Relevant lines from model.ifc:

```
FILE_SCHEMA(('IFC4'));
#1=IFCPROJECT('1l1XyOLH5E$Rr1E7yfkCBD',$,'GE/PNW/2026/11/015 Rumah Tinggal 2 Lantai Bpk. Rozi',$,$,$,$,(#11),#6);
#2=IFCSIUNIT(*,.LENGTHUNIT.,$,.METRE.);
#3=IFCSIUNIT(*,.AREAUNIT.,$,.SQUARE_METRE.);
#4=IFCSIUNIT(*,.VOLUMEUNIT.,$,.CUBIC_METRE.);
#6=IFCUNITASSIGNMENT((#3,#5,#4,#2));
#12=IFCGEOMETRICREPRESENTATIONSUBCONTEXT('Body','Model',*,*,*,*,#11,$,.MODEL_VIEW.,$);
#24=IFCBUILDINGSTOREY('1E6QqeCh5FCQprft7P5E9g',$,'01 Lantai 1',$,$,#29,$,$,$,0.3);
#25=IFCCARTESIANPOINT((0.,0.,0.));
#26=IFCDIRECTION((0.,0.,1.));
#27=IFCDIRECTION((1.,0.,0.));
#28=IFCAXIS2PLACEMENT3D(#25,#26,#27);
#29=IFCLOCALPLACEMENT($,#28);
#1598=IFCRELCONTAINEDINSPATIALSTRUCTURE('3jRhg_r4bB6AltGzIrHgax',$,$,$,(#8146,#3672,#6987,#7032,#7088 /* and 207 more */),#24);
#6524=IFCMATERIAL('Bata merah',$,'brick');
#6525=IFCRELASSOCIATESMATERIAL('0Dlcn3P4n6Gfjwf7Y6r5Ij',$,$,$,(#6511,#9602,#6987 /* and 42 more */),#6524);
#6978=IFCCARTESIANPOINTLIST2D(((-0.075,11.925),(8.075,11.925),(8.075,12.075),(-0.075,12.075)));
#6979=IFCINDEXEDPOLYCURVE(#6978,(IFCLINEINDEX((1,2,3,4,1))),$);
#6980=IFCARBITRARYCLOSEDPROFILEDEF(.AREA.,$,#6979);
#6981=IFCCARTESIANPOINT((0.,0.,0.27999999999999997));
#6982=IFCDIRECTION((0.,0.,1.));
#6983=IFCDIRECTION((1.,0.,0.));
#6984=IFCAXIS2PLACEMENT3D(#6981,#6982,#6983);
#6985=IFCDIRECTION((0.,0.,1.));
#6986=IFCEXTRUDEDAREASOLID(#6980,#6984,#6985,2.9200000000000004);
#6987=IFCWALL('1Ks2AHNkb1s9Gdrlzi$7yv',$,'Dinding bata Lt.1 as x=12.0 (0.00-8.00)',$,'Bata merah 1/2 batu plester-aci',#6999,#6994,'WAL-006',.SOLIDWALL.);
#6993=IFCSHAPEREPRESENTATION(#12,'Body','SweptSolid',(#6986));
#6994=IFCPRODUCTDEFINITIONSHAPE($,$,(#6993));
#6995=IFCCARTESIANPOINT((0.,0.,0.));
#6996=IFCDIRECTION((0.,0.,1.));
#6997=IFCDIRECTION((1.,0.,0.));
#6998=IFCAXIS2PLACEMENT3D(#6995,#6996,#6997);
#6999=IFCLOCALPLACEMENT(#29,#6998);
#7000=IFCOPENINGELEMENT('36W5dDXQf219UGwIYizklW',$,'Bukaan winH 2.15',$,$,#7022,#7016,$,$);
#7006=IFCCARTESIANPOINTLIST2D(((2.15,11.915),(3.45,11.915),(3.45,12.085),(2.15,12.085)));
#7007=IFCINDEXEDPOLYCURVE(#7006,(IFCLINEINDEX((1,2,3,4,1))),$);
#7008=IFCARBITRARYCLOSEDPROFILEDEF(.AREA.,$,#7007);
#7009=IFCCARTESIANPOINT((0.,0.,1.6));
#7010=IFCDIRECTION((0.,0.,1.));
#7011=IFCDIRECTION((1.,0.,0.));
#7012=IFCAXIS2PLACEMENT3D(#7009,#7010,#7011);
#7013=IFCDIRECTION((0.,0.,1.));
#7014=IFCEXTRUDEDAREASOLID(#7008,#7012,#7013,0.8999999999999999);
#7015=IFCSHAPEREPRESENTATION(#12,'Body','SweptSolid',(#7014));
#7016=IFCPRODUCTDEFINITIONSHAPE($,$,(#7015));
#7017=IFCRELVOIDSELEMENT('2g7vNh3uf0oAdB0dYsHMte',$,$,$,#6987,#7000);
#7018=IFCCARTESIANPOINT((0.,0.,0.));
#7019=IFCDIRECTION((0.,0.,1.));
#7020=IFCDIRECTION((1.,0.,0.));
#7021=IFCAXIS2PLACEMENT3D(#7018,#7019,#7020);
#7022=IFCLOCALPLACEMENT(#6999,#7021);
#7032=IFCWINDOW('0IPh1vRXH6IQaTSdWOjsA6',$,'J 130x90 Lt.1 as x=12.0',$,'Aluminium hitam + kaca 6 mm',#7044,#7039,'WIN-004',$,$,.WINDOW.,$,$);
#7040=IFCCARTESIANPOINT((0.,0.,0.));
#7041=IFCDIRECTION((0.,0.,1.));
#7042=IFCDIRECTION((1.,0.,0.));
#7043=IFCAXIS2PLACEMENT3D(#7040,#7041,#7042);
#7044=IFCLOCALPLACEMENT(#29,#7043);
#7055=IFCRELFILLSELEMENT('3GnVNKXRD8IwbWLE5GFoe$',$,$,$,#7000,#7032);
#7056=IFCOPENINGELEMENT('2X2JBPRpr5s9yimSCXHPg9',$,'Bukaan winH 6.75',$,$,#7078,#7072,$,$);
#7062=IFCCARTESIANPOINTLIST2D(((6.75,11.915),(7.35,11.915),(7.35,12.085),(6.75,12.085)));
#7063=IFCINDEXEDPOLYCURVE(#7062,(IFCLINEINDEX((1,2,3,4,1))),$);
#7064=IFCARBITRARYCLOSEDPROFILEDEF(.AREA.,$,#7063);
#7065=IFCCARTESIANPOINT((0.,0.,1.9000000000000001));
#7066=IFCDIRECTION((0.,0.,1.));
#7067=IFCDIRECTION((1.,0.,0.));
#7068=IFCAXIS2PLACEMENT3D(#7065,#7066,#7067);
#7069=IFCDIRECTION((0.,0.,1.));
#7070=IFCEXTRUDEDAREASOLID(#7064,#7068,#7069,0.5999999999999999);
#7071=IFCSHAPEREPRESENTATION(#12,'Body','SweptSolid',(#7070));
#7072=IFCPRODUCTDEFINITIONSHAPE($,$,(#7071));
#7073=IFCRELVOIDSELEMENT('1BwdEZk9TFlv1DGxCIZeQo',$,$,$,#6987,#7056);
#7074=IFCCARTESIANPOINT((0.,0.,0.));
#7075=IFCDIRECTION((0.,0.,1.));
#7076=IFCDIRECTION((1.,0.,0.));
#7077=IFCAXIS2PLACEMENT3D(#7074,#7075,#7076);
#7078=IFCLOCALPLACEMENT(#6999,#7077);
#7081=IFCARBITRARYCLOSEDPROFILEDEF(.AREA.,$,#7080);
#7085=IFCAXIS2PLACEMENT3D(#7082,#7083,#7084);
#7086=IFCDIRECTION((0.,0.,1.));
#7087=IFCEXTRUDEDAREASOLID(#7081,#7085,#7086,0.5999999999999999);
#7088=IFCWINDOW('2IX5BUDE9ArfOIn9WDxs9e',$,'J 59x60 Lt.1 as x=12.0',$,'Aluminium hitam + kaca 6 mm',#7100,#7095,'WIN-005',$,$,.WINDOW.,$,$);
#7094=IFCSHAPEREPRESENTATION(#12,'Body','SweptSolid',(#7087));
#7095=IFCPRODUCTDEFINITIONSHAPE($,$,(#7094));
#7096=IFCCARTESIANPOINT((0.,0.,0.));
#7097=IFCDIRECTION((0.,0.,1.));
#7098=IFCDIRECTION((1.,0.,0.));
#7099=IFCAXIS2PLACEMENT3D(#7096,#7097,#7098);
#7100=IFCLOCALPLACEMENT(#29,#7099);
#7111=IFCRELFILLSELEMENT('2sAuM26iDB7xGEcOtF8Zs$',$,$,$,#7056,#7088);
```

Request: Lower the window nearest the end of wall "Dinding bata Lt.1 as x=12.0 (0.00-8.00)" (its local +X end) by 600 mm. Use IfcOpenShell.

```python
import numpy as np
import ifcopenshell
import ifcopenshell.api.geometry
import ifcopenshell.util.placement
import ifcopenshell.util.unit

model = ifcopenshell.open("model.ifc")
unit_scale = ifcopenshell.util.unit.calculate_unit_scale(model)

window = model.by_guid("2IX5BUDE9ArfOIn9WDxs9e")
opening = window.FillsVoids[0].RelatingOpeningElement
dz = -0.6

shift = np.array([0.0, 0.0, dz])
# The window is not placed relative to its opening, so move both.
for product in (opening, window):
    matrix = ifcopenshell.util.placement.get_local_placement(product.ObjectPlacement)
    matrix[:3, 3] += shift
    ifcopenshell.api.geometry.edit_object_placement(model, product=product, matrix=matrix, is_si=False)

print(f"moved by {dz * unit_scale:+.3f} m")

model.write("model_v2.ifc")
```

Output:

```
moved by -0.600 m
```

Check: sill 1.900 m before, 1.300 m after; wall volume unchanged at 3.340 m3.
